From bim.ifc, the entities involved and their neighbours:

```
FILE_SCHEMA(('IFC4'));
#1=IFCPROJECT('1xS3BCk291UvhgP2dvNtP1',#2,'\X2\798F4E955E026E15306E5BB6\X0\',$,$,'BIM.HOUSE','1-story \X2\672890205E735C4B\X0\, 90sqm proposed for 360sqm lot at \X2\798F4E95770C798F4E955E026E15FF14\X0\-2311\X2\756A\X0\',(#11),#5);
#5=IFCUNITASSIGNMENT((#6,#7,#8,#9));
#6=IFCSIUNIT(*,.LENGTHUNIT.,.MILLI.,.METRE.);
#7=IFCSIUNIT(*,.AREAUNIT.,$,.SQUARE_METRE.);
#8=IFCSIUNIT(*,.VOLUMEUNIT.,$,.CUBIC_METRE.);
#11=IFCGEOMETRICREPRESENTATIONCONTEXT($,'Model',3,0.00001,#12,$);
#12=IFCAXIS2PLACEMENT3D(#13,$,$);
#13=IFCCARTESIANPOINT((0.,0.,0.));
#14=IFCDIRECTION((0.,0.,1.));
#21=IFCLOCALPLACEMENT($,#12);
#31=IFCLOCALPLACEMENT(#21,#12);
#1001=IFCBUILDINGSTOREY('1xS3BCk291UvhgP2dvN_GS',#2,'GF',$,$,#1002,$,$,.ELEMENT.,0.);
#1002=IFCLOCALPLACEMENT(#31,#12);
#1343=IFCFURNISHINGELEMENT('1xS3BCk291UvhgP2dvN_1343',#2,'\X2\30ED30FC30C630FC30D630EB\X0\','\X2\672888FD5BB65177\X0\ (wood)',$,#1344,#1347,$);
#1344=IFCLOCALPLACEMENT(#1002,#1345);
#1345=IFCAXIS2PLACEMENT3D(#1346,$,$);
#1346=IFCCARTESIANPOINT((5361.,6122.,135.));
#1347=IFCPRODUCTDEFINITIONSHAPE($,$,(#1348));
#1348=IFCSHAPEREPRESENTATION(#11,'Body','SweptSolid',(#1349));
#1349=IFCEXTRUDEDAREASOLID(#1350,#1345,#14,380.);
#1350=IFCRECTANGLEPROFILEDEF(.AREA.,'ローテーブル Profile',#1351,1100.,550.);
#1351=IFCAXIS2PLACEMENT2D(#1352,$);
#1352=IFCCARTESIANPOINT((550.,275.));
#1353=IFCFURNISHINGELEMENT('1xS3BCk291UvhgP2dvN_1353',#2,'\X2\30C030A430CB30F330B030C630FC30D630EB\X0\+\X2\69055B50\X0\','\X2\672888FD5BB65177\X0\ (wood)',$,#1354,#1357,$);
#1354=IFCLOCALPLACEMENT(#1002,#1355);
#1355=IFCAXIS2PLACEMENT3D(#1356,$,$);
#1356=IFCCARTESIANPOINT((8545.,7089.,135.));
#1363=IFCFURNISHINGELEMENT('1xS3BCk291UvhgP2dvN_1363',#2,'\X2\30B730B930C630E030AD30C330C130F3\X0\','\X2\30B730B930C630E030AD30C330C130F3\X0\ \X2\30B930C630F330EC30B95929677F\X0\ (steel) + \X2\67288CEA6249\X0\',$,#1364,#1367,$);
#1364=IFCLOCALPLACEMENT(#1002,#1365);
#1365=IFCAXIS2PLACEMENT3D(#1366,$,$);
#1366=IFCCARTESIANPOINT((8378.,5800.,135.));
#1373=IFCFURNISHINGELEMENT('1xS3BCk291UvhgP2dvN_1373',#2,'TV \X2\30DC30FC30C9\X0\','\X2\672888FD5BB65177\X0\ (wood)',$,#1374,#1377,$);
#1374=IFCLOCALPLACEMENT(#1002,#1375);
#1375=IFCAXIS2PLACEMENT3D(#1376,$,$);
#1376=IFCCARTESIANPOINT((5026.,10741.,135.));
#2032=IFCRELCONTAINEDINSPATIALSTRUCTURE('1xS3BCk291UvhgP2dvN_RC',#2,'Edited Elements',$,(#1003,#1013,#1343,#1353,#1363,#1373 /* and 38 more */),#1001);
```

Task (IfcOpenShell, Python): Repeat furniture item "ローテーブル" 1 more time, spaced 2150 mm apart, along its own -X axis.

```python
import ifcopenshell
import ifcopenshell.api.geometry
import ifcopenshell.api.root
import ifcopenshell.util.element
import ifcopenshell.util.placement
import ifcopenshell.util.unit

model = ifcopenshell.open("bim.ifc")
unit_scale = ifcopenshell.util.unit.calculate_unit_scale(model)


def reuse_history(source, copy):
    """copy_class also copies each property set's owner history, people and application; keep the originals."""
    for rel in copy.IsDefinedBy:
        if rel.is_a("IfcRelDefinesByProperties") and (history := rel.RelatingPropertyDefinition.OwnerHistory):
            rel.RelatingPropertyDefinition.OwnerHistory = source.OwnerHistory
            ifcopenshell.util.element.remove_deep2(model, history)


source = model.by_id(1343)
base = ifcopenshell.util.placement.get_local_placement(source.ObjectPlacement)
step = -base[:3, 0] * 2.15 / unit_scale

for i in range(1, 2):
    copy = ifcopenshell.api.root.copy_class(model, product=source)
    copy.Representation = ifcopenshell.util.element.copy_deep(
        model, source.Representation, exclude=["IfcGeometricRepresentationContext", "IfcRepresentationMap"]
    )
    reuse_history(source, copy)
    matrix = base.copy()
    matrix[:3, 3] += i * step
    print("added at", matrix[:3, 3].round(3) + 0.0)
    ifcopenshell.api.geometry.edit_object_placement(model, product=copy, matrix=matrix, is_si=False)

model.write("bim_edited.ifc")
```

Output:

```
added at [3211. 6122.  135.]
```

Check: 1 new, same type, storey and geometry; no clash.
